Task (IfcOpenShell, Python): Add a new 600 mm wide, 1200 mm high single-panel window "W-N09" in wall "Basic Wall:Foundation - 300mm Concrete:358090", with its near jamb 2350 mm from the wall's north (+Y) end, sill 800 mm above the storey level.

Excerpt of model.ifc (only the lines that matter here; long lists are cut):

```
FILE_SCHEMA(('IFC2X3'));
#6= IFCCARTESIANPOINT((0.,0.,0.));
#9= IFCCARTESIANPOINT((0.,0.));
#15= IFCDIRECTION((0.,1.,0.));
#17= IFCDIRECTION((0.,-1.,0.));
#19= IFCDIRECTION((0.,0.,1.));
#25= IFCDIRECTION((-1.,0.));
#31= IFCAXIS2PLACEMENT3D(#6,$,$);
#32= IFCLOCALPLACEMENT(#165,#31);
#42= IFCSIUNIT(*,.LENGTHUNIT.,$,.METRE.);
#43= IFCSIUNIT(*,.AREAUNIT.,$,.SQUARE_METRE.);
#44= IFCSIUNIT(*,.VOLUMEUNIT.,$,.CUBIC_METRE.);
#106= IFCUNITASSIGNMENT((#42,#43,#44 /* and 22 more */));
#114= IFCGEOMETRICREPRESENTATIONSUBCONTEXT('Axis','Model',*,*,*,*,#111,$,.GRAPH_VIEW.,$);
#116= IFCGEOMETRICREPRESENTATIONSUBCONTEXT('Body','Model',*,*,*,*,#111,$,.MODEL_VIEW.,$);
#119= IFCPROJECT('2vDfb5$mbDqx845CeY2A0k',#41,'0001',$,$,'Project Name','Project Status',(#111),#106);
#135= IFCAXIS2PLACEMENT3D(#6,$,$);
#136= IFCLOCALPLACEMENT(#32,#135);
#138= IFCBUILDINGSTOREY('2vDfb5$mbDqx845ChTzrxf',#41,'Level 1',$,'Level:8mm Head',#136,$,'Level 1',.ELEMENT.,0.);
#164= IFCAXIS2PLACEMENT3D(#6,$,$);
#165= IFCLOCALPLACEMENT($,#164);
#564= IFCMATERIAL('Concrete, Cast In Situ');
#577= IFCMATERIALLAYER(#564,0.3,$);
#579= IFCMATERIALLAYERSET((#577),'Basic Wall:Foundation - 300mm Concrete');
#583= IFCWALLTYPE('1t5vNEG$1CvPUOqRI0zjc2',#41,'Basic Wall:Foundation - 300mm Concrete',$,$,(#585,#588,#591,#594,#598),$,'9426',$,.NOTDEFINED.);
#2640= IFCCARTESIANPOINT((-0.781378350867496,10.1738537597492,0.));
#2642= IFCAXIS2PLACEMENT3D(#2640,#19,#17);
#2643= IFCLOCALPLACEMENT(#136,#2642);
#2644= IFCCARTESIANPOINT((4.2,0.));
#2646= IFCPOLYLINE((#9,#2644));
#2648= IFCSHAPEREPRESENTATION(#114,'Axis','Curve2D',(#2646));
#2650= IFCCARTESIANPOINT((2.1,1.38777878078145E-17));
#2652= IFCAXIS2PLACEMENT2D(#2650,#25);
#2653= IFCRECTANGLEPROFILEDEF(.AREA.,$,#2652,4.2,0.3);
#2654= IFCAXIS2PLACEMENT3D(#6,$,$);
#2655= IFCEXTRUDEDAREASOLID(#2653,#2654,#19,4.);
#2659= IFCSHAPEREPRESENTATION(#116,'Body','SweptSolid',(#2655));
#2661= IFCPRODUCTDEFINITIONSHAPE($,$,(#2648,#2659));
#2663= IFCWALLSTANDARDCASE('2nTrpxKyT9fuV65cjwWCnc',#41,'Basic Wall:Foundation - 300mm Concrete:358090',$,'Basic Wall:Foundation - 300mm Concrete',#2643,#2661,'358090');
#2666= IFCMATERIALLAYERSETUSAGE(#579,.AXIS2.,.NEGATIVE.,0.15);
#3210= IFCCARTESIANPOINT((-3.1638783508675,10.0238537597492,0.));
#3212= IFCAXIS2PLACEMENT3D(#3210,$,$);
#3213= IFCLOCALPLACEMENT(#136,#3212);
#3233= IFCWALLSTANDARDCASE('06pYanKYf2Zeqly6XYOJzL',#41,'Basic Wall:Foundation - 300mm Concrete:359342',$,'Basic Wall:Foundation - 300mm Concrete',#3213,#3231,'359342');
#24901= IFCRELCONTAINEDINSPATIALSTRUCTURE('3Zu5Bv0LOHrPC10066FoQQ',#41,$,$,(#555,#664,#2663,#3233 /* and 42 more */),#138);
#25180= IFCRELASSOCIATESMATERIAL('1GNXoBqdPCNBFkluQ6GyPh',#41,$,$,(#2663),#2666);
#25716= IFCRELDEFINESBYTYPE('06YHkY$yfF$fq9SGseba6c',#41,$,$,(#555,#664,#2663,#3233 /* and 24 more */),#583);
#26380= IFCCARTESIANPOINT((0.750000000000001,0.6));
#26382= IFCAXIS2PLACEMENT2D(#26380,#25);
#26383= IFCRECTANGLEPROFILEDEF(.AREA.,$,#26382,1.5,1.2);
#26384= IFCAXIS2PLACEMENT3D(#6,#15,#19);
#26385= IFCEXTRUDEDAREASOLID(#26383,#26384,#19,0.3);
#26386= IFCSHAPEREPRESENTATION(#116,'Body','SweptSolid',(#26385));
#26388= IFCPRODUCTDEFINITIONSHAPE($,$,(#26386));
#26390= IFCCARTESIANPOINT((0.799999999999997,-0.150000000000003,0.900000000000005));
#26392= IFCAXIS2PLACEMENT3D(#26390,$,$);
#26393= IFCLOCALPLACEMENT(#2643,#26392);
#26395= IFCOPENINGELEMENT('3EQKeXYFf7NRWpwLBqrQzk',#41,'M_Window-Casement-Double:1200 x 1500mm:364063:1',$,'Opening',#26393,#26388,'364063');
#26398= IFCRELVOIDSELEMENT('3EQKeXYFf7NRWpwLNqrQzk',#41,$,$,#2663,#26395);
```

```python
import numpy as np
import ifcopenshell
import ifcopenshell.api.feature
import ifcopenshell.api.geometry
import ifcopenshell.api.root
import ifcopenshell.api.spatial
import ifcopenshell.api.type
import ifcopenshell.geom
import ifcopenshell.util.element
import ifcopenshell.util.placement
import ifcopenshell.util.representation
import ifcopenshell.util.shape
import ifcopenshell.util.unit

model = ifcopenshell.open("model.ifc")
unit_scale = ifcopenshell.util.unit.calculate_unit_scale(model)
settings = ifcopenshell.geom.settings()


def volume(element):
    """Net volume in cubic metres, openings subtracted."""
    shape = ifcopenshell.geom.create_shape(settings, element)
    return ifcopenshell.util.shape.get_volume(shape.geometry)


wall = model.by_guid("2nTrpxKyT9fuV65cjwWCnc")
storey = ifcopenshell.util.element.get_container(wall, ifc_class="IfcBuildingStorey")
context = ifcopenshell.util.representation.get_context(model, "Model", "Body", "MODEL_VIEW")
before = volume(wall)

width, height, from_end, sill = 0.6, 1.2, 2.35, 0.8  # metres

# The wall runs along its own X axis, and the end named is its -X end.
wall_shape = ifcopenshell.geom.create_shape(settings, wall)
x, y, z = ifcopenshell.util.shape.get_vertices(wall_shape.geometry).T
start = x.min() + from_end
face, thickness = float(y.min()), float(y.max() - y.min())
wall_matrix = ifcopenshell.util.placement.get_local_placement(wall.ObjectPlacement)
level = ifcopenshell.util.placement.get_local_placement(storey.ObjectPlacement)[2, 3]


def in_wall(x, y):
    """Placement at x, y metres in the wall's axes, at sill height."""
    matrix = wall_matrix.copy()
    matrix[:, 3] = wall_matrix @ np.array([x / unit_scale, y / unit_scale, 0.0, 1.0])
    matrix[2, 3] = level + sill / unit_scale
    return matrix


# Opening: a box that overshoots both wall faces by 50 mm.
opening = ifcopenshell.api.root.create_entity(model, ifc_class="IfcOpeningElement")
box = ifcopenshell.api.geometry.add_wall_representation(
    model, context=context, length=width, height=height, thickness=thickness + 0.1
)
ifcopenshell.api.geometry.assign_representation(model, product=opening, representation=box)
ifcopenshell.api.geometry.edit_object_placement(model, product=opening, matrix=in_wall(start, face - 0.05), is_si=False)
ifcopenshell.api.feature.add_feature(model, feature=opening, element=wall)

window = ifcopenshell.api.root.create_entity(model, ifc_class="IfcWindow", name="W-N09")
window.OverallWidth, window.OverallHeight = width / unit_scale, height / unit_scale
body = ifcopenshell.api.geometry.add_window_representation(
    model,
    context=context,
    overall_width=window.OverallWidth,
    overall_height=window.OverallHeight,
    partition_type="SINGLE_PANEL",
)
ifcopenshell.api.geometry.assign_representation(model, product=window, representation=body)
ifcopenshell.api.spatial.assign_container(model, products=[window], relating_structure=storey)
fills = ifcopenshell.api.feature.add_filling(model, opening=opening, element=window)
fills.OwnerHistory = window.OwnerHistory  # required in IFC2X3

# IFC2X3 keeps the operation on the window style.
style = ifcopenshell.api.root.create_entity(model, ifc_class="IfcWindowStyle", name="W-N09")
style.OperationType, style.ConstructionType = "SINGLE_PANEL", "NOTDEFINED"
style.ParameterTakesPrecedence = style.Sizeable = False
ifcopenshell.api.type.assign_type(model, related_objects=[window], relating_type=style)

# Centre the window in the wall's thickness.
ifcopenshell.api.geometry.edit_object_placement(model, product=window, matrix=in_wall(start, face), is_si=False)
window_shape = ifcopenshell.geom.create_shape(settings, window)
depth = ifcopenshell.util.shape.get_vertices(window_shape.geometry)[:, 1]
offset = face + thickness / 2 - (depth.min() + depth.max()) / 2
ifcopenshell.api.geometry.edit_object_placement(model, product=window, matrix=in_wall(start, offset), is_si=False)

after = volume(wall)

print(f"wall volume {before:.3f} -> {after:.3f} m3")

model.write("model_v2.ifc")
```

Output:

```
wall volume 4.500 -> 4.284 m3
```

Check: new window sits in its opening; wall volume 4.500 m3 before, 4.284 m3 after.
